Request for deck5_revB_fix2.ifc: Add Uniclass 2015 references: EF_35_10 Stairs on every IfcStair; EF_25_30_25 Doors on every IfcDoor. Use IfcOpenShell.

First a look at what the model holds.

```python
import ifcopenshell

model = ifcopenshell.open("deck5_revB_fix2.ifc")
print(model.schema)
print("classifications:", [c.Name for c in model.by_type("IfcClassification")])
for ifc_class in ("IfcDoor", "IfcRoof", "IfcStair", "IfcWall", "IfcWindow"):
    print(ifc_class, len(model.by_type(ifc_class)))
```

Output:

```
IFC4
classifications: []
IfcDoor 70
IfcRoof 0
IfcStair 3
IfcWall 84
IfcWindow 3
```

```python
import ifcopenshell
import ifcopenshell.api.classification

model = ifcopenshell.open("deck5_revB_fix2.ifc")

system = ifcopenshell.api.classification.add_classification(model, classification="Uniclass 2015")

codes = {
    "IfcStair": ("EF_35_10", "Stairs"),
    "IfcDoor": ("EF_25_30_25", "Doors"),
}
for ifc_class, (code, name) in codes.items():
    products = model.by_type(ifc_class)
    ifcopenshell.api.classification.add_reference(
        model, products=products, classification=system, identification=code, name=name
    )
    print(code, len(products))

model.write("deck5_revB_fix2_updated.ifc")
```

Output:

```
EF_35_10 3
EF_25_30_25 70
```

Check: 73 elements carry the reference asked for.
